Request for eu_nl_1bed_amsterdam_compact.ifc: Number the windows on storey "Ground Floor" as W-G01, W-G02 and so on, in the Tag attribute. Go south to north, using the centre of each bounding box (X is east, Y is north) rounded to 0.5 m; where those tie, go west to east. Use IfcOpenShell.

First a look at what the model holds.

```python
import ifcopenshell
import ifcopenshell.util.element
import ifcopenshell.util.placement

model = ifcopenshell.open("eu_nl_1bed_amsterdam_compact.ifc")
print(model.schema)
storey = next(s for s in model.by_type("IfcBuildingStorey") if s.Name == "Ground Floor")
windows = [e for e in ifcopenshell.util.element.get_decomposition(storey) if e.is_a("IfcWindow")]
for e in sorted(windows, key=lambda e: e.id()):
    origin = ifcopenshell.util.placement.get_local_placement(e.ObjectPlacement)[:3, 3]
    print(e.id(), e.Tag, e.Name, origin.round(2) + 0.0, sep=" | ")
```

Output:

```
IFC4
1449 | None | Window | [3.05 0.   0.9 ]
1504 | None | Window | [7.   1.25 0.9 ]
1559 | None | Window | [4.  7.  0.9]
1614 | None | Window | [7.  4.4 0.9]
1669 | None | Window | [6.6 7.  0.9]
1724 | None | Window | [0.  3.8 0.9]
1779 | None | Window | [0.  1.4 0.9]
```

```python
import ifcopenshell
import ifcopenshell.geom
import ifcopenshell.util.element
import ifcopenshell.util.shape

model = ifcopenshell.open("eu_nl_1bed_amsterdam_compact.ifc")
settings = ifcopenshell.geom.settings()
settings.set("use-world-coords", True)


def centre(element):
    shape = ifcopenshell.geom.create_shape(settings, element)
    return ifcopenshell.util.shape.get_bbox_centroid(shape.geometry)


storey = next(s for s in model.by_type("IfcBuildingStorey") if s.Name == "Ground Floor")
windows = [e for e in ifcopenshell.util.element.get_decomposition(storey) if e.is_a("IfcWindow")]

# Insertion points can sit at a corner or the storey origin, so sort by the geometry (in metres).
centres = {e: centre(e) for e in windows}
windows.sort(key=lambda e: (round(centres[e][1] / 0.5), centres[e][0]))

for i, e in enumerate(windows, start=1):
    number = f"W-G{i:02d}"
    e.Tag = number
    print(e.id(), number)

model.write("eu_nl_1bed_amsterdam_compact_rev.ifc")
```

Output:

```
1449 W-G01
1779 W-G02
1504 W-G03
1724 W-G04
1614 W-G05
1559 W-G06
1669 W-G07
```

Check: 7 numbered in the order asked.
